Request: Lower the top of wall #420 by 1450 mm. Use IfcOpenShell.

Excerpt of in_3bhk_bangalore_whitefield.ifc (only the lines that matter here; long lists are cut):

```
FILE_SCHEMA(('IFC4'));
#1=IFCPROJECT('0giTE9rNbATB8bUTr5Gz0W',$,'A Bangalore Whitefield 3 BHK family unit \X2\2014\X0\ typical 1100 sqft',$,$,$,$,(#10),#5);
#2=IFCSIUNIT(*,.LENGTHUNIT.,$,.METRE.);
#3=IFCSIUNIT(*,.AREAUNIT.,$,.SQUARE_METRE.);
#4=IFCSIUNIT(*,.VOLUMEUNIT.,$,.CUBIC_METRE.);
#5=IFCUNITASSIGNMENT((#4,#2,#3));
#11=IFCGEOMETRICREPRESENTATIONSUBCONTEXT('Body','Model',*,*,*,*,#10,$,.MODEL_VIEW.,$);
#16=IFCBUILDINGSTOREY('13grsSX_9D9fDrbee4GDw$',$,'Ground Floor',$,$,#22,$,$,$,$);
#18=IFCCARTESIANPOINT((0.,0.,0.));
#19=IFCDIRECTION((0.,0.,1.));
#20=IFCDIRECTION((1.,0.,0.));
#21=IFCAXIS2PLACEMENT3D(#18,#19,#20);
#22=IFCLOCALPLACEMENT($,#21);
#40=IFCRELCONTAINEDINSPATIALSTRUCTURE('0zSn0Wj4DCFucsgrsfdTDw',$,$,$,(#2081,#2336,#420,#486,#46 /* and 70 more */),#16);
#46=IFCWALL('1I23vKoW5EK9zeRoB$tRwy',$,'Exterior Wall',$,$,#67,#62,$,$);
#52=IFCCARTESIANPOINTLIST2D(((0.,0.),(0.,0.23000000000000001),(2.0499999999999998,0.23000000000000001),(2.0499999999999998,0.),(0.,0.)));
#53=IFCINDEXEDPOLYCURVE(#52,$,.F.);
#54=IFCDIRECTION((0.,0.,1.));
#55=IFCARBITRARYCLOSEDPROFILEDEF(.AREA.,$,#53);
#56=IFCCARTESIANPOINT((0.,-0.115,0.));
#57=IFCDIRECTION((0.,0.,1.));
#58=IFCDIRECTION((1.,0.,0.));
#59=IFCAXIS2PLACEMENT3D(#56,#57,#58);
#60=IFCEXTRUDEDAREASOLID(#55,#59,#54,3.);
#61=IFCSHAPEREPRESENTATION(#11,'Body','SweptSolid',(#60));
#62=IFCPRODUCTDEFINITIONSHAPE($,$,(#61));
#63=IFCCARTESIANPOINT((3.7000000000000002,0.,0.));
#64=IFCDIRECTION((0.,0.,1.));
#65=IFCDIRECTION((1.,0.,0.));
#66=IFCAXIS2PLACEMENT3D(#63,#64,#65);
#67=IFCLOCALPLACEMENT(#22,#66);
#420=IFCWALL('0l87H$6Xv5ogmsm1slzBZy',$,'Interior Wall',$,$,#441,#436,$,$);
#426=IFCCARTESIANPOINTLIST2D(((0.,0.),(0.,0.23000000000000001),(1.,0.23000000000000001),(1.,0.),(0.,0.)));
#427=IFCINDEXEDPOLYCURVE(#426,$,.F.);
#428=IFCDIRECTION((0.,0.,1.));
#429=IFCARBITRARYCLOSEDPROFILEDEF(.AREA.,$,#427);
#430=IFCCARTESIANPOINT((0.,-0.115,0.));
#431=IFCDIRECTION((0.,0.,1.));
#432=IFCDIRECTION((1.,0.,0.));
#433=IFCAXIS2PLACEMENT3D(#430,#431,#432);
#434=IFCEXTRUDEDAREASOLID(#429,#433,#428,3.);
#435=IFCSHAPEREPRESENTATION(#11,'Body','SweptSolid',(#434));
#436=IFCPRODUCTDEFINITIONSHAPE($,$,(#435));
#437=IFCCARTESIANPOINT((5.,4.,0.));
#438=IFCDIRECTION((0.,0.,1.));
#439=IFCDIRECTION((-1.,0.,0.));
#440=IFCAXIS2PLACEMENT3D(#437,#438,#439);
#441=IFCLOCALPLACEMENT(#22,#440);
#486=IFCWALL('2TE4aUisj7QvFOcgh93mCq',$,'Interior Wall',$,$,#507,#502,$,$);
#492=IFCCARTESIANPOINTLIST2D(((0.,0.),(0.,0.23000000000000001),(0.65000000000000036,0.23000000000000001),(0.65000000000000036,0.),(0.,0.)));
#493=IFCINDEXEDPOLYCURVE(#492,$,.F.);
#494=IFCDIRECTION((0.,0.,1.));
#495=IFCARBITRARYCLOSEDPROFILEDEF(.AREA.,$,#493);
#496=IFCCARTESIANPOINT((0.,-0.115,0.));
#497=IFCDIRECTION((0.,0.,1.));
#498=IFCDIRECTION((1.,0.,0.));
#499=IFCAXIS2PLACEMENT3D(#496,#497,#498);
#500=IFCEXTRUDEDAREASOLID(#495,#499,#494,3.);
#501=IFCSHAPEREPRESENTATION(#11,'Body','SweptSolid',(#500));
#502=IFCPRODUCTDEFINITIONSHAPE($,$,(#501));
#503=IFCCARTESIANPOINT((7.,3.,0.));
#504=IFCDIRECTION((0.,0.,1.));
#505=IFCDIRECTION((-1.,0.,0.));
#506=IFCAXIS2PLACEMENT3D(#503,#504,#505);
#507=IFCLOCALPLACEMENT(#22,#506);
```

```python
import ifcopenshell
import ifcopenshell.geom
import ifcopenshell.util.representation
import ifcopenshell.util.shape

model = ifcopenshell.open("in_3bhk_bangalore_whitefield.ifc")
settings = ifcopenshell.geom.settings()


def volume(element):
    """Net volume in cubic metres, openings subtracted."""
    shape = ifcopenshell.geom.create_shape(settings, element)
    return ifcopenshell.util.shape.get_volume(shape.geometry)


wall = model.by_guid("0l87H$6Xv5ogmsm1slzBZy")
before = volume(wall)

body = ifcopenshell.util.representation.get_representation(wall, "Model", "Body")
solid = body.Items[0]
old_height = solid.Depth
solid.Depth -= 1.45
after = volume(wall)

print(f"height {old_height:g} -> {solid.Depth:g}, volume {before:.3f} -> {after:.3f} m3")

model.write("in_3bhk_bangalore_whitefield-out.ifc")
```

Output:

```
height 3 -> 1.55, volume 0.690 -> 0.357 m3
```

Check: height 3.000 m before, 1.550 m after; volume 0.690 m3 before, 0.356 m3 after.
